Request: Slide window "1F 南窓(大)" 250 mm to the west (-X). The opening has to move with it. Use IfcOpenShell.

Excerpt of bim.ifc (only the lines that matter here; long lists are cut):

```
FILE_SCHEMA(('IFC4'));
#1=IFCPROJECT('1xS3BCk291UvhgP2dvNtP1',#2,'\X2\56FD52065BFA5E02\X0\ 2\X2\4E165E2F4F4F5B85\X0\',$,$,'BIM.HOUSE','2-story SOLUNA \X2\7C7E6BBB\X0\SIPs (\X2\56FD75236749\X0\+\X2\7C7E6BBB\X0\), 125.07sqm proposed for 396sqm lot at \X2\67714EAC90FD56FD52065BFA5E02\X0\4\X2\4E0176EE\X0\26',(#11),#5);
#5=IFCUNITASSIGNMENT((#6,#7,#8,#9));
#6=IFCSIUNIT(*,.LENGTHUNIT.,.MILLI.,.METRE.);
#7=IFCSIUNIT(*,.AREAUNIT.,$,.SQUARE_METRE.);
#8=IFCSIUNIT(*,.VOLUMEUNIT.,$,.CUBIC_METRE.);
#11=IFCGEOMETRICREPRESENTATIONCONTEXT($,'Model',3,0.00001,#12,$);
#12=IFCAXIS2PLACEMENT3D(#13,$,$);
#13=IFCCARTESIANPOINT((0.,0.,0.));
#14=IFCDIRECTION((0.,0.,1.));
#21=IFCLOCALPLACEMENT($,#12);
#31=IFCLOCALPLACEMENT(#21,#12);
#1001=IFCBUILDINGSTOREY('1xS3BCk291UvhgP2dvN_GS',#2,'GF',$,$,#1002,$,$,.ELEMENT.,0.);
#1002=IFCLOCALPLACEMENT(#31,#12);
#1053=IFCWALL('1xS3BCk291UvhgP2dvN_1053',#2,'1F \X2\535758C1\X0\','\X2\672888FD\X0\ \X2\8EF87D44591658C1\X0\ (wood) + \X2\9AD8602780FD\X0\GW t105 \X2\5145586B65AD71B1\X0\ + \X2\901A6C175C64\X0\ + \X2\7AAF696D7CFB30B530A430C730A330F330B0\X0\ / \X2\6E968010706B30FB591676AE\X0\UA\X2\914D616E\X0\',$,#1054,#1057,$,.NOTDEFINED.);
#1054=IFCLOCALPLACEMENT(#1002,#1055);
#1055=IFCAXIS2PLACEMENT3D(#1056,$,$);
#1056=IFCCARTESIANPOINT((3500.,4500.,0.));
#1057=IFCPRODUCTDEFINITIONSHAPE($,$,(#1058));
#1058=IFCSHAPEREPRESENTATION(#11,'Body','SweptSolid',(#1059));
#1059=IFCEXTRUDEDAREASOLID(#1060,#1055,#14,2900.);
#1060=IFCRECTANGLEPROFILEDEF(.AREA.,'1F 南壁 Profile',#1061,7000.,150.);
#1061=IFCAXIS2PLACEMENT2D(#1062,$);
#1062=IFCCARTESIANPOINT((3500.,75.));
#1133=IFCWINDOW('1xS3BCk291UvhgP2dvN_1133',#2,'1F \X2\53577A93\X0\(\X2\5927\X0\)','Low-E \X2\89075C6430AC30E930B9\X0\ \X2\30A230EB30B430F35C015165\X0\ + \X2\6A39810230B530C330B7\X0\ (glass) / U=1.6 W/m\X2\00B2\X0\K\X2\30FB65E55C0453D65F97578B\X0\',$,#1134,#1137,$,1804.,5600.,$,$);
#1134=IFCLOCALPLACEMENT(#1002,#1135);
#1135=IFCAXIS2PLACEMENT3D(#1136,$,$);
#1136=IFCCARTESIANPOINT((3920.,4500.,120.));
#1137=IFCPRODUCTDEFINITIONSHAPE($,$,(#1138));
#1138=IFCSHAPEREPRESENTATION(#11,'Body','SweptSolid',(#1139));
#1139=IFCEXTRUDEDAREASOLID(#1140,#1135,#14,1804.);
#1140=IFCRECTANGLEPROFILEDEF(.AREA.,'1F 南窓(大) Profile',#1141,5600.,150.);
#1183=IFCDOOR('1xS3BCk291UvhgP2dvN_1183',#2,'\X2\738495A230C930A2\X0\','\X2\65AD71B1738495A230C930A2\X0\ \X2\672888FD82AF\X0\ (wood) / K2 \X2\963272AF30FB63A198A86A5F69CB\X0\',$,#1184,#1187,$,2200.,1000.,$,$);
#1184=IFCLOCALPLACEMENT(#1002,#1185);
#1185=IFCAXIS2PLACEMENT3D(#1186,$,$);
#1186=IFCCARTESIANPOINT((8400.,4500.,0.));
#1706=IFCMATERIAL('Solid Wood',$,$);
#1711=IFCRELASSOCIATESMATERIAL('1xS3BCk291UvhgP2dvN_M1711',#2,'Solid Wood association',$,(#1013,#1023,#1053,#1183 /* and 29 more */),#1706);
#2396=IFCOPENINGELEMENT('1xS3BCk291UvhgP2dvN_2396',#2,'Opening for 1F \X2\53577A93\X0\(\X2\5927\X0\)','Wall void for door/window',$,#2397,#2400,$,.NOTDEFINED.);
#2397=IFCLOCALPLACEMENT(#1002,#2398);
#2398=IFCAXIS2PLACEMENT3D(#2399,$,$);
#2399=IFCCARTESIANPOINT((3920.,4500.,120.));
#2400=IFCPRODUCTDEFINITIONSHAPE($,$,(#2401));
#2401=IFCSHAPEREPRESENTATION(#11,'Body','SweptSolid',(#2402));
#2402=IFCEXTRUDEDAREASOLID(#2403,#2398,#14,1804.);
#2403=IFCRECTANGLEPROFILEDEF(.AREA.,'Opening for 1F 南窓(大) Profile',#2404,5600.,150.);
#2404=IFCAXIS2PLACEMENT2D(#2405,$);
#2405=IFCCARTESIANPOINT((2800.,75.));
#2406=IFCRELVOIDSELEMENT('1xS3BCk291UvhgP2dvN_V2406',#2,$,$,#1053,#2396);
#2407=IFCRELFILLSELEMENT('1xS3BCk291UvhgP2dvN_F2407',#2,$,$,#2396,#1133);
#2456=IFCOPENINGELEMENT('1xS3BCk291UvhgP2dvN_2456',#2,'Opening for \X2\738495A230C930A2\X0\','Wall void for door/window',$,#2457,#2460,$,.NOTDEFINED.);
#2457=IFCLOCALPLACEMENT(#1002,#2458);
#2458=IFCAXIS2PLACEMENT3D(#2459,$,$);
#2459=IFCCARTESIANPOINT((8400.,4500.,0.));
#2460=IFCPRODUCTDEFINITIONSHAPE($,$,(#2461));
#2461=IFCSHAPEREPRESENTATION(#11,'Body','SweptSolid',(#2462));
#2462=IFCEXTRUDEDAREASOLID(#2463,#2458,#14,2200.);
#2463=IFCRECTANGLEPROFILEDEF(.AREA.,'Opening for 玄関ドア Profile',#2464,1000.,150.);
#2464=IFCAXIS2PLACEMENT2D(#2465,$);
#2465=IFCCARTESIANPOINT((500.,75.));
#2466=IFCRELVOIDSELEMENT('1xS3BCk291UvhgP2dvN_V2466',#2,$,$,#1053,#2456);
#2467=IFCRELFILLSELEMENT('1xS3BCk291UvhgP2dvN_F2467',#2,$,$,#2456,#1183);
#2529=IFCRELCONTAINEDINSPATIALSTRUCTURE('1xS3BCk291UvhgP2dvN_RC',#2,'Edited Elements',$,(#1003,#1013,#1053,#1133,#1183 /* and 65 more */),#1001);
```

```python
import ifcopenshell
import ifcopenshell.api.geometry
import ifcopenshell.util.placement

model = ifcopenshell.open("bim.ifc")

window = model.by_guid("1xS3BCk291UvhgP2dvN_1133")
opening = window.FillsVoids[0].RelatingOpeningElement
wall = opening.VoidsElements[0].RelatingBuildingElement

wall_matrix = ifcopenshell.util.placement.get_local_placement(wall.ObjectPlacement)
shift = wall_matrix[:3, 0] * -250.0
before = ifcopenshell.util.placement.get_local_placement(window.ObjectPlacement)[:3, 3].copy()

# The window is not placed relative to its opening, so move both.
for product in (opening, window):
    matrix = ifcopenshell.util.placement.get_local_placement(product.ObjectPlacement)
    matrix[:3, 3] += shift
    ifcopenshell.api.geometry.edit_object_placement(model, product=product, matrix=matrix, is_si=False)

after = ifcopenshell.util.placement.get_local_placement(window.ObjectPlacement)[:3, 3]
print("window moved by", (after - before).round(3) + 0.0)

model.write("bim_updated.ifc")
```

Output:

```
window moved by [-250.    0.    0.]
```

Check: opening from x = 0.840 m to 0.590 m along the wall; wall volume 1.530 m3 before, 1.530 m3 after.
